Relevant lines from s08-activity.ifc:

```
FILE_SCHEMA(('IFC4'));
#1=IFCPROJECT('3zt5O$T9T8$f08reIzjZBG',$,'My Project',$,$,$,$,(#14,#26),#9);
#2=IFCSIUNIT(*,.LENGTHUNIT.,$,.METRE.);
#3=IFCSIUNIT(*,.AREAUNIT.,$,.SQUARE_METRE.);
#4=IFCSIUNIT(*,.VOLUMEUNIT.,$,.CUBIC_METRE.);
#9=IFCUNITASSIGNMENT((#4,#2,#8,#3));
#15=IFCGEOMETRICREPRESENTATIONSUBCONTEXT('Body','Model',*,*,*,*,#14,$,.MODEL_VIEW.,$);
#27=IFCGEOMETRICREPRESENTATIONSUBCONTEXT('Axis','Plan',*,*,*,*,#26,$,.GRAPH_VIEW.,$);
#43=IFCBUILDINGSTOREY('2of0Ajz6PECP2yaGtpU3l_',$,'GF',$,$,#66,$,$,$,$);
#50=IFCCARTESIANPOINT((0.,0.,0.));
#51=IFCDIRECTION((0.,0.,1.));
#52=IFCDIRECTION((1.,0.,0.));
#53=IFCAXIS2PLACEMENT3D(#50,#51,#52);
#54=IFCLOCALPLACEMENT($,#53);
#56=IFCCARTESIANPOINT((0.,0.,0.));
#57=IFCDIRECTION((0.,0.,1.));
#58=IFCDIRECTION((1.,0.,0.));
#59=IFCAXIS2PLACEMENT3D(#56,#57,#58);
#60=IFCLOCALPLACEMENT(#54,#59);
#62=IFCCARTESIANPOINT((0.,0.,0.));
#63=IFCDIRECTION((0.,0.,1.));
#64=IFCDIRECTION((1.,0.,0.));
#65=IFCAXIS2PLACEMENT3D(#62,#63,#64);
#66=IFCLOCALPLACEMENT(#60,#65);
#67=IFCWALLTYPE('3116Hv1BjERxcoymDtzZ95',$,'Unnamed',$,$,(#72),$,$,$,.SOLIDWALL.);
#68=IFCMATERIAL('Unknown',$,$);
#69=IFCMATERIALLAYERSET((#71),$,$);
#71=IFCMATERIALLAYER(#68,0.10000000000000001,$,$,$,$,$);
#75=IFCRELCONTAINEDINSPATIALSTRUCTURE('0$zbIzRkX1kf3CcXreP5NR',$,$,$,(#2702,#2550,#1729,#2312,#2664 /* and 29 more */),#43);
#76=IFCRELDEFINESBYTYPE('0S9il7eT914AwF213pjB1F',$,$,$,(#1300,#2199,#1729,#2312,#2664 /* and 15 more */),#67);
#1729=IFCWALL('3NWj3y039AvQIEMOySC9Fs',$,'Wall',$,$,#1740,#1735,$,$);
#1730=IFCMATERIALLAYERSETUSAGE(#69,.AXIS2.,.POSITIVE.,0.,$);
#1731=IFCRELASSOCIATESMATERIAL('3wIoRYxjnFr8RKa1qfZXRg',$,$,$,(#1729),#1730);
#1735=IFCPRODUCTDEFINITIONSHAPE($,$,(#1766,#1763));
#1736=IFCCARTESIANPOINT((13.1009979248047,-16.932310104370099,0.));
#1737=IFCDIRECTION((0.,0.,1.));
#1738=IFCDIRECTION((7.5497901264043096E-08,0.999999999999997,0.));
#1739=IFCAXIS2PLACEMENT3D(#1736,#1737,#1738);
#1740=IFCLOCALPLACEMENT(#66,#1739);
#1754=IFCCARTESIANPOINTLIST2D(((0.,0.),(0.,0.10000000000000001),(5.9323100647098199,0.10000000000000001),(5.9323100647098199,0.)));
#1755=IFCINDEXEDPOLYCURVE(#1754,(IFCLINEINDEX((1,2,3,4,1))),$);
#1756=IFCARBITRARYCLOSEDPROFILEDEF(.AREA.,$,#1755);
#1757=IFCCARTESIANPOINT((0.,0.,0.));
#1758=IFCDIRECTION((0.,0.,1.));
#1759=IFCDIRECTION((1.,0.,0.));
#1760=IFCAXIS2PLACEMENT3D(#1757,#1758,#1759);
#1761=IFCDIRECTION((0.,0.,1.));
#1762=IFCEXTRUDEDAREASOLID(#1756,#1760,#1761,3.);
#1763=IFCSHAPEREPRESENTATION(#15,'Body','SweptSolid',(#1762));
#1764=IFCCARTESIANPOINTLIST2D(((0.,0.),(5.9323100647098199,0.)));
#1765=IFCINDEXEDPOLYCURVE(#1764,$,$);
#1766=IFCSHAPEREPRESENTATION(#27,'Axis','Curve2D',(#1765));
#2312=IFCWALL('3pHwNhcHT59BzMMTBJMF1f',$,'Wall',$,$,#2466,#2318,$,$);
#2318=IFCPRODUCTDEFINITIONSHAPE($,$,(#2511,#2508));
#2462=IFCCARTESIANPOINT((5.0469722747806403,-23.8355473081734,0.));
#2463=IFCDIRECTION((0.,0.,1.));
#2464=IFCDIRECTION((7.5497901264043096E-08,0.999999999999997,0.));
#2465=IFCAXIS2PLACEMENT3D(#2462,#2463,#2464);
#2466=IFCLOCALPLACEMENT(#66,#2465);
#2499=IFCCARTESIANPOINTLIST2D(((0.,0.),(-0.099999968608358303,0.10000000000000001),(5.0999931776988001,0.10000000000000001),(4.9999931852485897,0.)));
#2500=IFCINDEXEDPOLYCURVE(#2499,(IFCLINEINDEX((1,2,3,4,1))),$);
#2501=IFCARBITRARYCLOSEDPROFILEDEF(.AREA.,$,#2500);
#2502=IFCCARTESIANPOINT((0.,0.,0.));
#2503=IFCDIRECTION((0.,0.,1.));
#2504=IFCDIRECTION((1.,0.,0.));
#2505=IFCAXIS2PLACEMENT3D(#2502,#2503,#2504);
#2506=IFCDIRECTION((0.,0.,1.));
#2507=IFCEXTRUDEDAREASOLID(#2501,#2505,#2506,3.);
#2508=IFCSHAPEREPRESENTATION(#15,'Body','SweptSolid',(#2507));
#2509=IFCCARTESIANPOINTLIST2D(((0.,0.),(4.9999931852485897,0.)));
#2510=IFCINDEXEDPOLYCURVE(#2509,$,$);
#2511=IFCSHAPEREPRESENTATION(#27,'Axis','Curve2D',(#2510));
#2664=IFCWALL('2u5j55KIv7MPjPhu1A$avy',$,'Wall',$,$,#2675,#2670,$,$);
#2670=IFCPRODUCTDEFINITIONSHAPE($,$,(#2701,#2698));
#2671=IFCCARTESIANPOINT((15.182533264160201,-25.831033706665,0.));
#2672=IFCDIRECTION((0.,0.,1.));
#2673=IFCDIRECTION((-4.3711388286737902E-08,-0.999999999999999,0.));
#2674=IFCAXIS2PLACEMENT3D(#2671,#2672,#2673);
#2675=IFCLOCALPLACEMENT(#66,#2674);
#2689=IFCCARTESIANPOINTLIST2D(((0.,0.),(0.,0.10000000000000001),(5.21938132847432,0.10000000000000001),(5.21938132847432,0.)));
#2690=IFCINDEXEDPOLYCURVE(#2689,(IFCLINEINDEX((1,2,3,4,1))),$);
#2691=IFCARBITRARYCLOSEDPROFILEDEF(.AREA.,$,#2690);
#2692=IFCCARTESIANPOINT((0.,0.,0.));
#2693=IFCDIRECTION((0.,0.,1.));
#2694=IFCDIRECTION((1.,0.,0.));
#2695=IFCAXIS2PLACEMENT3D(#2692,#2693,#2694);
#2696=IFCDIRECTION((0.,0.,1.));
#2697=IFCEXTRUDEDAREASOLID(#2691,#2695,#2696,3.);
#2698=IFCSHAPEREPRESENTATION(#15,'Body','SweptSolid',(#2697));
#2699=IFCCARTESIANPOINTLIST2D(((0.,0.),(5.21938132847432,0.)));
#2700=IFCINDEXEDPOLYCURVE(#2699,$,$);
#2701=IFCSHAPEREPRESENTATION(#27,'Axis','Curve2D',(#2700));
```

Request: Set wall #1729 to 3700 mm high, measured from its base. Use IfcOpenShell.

```python
import ifcopenshell
import ifcopenshell.geom
import ifcopenshell.util.representation
import ifcopenshell.util.shape

model = ifcopenshell.open("s08-activity.ifc")
settings = ifcopenshell.geom.settings()


def volume(element):
    """Net volume in cubic metres, openings subtracted."""
    shape = ifcopenshell.geom.create_shape(settings, element)
    return ifcopenshell.util.shape.get_volume(shape.geometry)


wall = model.by_guid("3NWj3y039AvQIEMOySC9Fs")
before = volume(wall)

body = ifcopenshell.util.representation.get_representation(wall, "Model", "Body")
solid = body.Items[0]
old_height = solid.Depth
solid.Depth = 3.7
after = volume(wall)

print(f"height {old_height:g} -> {solid.Depth:g}, volume {before:.3f} -> {after:.3f} m3")

model.write("s08-activity_v2.ifc")
```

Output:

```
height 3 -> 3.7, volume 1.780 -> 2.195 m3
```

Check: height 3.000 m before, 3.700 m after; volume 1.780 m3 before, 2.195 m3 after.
